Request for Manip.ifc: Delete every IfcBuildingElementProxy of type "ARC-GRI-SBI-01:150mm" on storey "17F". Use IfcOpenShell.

First a look at what the model holds.

```python
import ifcopenshell
import ifcopenshell.util.element

model = ifcopenshell.open("Manip.ifc")
print(model.schema)
storey = next(s for s in model.by_type("IfcBuildingStorey") if s.Name == "17F")
proxies = [e for e in ifcopenshell.util.element.get_decomposition(storey) if e.is_a("IfcBuildingElementProxy")]
seen = {}
for e in proxies:
    element_type = ifcopenshell.util.element.get_type(e)
    name = element_type.Name if element_type not in (None, e) else None
    seen[name] = seen.get(name, 0) + 1
for name, count in sorted(seen.items(), key=str):
    print(count, "x", name)
```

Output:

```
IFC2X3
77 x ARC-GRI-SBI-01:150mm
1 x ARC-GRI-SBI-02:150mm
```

```python
import ifcopenshell
import ifcopenshell.api.root
import ifcopenshell.util.element

model = ifcopenshell.open("Manip.ifc")

storey = next(s for s in model.by_type("IfcBuildingStorey") if s.Name == "17F")
proxies = [e for e in ifcopenshell.util.element.get_decomposition(storey) if e.is_a("IfcBuildingElementProxy")]
targets = [e for e in proxies if (t := ifcopenshell.util.element.get_type(e)) not in (None, e) and t.Name == "ARC-GRI-SBI-01:150mm"]

for e in targets:
    ifcopenshell.api.root.remove_product(model, product=e)
print(len(targets), "removed")

model.write("Manip_edited.ifc")
```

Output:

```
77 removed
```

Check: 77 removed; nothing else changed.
